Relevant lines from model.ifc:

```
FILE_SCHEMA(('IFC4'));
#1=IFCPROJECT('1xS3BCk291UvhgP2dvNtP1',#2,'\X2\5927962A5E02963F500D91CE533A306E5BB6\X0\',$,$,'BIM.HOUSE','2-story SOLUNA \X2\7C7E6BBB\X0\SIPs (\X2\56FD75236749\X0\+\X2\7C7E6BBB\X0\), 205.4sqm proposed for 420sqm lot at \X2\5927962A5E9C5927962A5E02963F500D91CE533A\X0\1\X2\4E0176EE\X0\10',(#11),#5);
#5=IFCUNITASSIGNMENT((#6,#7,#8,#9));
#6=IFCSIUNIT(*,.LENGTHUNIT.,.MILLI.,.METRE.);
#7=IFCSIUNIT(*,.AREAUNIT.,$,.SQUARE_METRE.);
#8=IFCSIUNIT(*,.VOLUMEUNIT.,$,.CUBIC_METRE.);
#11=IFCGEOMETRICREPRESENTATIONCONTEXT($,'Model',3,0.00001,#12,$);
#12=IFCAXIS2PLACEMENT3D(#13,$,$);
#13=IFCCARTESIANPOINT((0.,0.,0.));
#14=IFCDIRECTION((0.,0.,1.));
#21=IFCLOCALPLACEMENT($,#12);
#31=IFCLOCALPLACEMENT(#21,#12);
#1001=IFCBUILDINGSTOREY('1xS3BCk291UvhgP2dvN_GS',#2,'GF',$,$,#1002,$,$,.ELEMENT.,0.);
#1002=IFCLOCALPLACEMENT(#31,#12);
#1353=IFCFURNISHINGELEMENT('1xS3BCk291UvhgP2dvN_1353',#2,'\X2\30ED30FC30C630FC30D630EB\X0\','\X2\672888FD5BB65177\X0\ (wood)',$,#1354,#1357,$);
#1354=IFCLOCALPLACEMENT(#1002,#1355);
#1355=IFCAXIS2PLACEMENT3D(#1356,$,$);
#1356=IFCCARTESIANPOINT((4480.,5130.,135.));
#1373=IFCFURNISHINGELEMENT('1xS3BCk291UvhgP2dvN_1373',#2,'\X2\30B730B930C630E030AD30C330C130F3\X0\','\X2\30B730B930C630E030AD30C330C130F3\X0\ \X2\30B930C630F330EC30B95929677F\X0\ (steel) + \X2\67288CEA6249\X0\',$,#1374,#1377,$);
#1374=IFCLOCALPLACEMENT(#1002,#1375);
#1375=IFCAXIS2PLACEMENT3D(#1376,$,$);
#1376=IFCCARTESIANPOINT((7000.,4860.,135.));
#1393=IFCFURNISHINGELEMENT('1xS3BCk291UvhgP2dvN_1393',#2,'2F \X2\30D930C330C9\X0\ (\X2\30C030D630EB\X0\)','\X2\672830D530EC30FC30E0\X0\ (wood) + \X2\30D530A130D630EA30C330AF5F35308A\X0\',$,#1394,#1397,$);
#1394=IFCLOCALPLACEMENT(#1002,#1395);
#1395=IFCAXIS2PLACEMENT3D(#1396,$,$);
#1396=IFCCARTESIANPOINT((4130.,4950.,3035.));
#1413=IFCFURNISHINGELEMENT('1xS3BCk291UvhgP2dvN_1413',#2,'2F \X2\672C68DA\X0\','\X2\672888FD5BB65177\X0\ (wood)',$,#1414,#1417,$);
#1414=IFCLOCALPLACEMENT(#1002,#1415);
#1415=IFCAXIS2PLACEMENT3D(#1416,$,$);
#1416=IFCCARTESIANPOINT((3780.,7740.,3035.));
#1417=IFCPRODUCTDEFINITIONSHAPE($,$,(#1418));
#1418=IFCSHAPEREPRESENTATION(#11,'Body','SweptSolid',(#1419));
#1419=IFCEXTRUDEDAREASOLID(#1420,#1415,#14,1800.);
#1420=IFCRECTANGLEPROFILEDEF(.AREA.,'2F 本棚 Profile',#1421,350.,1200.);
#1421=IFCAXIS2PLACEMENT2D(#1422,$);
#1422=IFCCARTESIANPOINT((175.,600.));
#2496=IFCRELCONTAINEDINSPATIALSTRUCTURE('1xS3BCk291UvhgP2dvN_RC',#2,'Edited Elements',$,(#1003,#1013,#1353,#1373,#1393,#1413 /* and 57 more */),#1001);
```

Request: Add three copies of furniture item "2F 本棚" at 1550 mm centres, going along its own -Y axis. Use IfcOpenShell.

```python
import ifcopenshell
import ifcopenshell.api.geometry
import ifcopenshell.api.root
import ifcopenshell.util.element
import ifcopenshell.util.placement
import ifcopenshell.util.unit

model = ifcopenshell.open("model.ifc")
unit_scale = ifcopenshell.util.unit.calculate_unit_scale(model)


def reuse_history(source, copy):
    """copy_class also copies each property set's owner history, people and application; keep the originals."""
    for rel in copy.IsDefinedBy:
        if rel.is_a("IfcRelDefinesByProperties") and (history := rel.RelatingPropertyDefinition.OwnerHistory):
            rel.RelatingPropertyDefinition.OwnerHistory = source.OwnerHistory
            ifcopenshell.util.element.remove_deep2(model, history)


source = model.by_guid("1xS3BCk291UvhgP2dvN_1413")
base = ifcopenshell.util.placement.get_local_placement(source.ObjectPlacement)
step = -base[:3, 1] * 1.55 / unit_scale

for i in range(1, 4):
    copy = ifcopenshell.api.root.copy_class(model, product=source)
    copy.Representation = ifcopenshell.util.element.copy_deep(
        model, source.Representation, exclude=["IfcGeometricRepresentationContext", "IfcRepresentationMap"]
    )
    reuse_history(source, copy)
    matrix = base.copy()
    matrix[:3, 3] += i * step
    print("added at", matrix[:3, 3].round(3) + 0.0)
    ifcopenshell.api.geometry.edit_object_placement(model, product=copy, matrix=matrix, is_si=False)

model.write("model_v2.ifc")
```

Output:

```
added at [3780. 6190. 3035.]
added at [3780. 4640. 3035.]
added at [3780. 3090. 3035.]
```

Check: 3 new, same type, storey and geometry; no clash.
